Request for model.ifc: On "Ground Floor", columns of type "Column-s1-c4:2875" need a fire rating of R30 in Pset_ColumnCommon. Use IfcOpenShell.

First a look at what the model holds.

```python
import ifcopenshell
import ifcopenshell.util.element

model = ifcopenshell.open("model.ifc")
print(model.schema)
storey = next(s for s in model.by_type("IfcBuildingStorey") if s.Name == "Ground Floor")
columns = [e for e in ifcopenshell.util.element.get_decomposition(storey) if e.is_a("IfcColumn")]
seen = {}
for e in columns:
    element_type = ifcopenshell.util.element.get_type(e)
    key = (element_type.Name if element_type != e and element_type else None, ifcopenshell.util.element.get_pset(e, "Pset_ColumnCommon", "FireRating"))
    seen[key] = seen.get(key, 0) + 1
for (name, value), count in sorted(seen.items(), key=str):
    print(count, "x", name, "|", value)
```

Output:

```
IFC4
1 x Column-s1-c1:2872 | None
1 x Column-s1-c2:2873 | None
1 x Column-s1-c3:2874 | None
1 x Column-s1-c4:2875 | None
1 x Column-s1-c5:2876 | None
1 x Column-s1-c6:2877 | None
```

```python
import ifcopenshell
import ifcopenshell.api.pset
import ifcopenshell.util.element

model = ifcopenshell.open("model.ifc")

storey = next(s for s in model.by_type("IfcBuildingStorey") if s.Name == "Ground Floor")
columns = [e for e in ifcopenshell.util.element.get_decomposition(storey) if e.is_a("IfcColumn")]

count = 0
for e in columns:
    element_type = ifcopenshell.util.element.get_type(e)
    if element_type in (None, e) or element_type.Name != "Column-s1-c4:2875":
        continue
    # add_pset returns the element's existing set when there is one.
    pset = ifcopenshell.api.pset.add_pset(model, product=e, name="Pset_ColumnCommon")
    ifcopenshell.api.pset.edit_pset(model, pset=pset, properties={"FireRating": "R30"})
    count += 1

print(count, "columns updated")

model.write("model_v2.ifc")
```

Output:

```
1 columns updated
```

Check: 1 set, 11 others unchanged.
